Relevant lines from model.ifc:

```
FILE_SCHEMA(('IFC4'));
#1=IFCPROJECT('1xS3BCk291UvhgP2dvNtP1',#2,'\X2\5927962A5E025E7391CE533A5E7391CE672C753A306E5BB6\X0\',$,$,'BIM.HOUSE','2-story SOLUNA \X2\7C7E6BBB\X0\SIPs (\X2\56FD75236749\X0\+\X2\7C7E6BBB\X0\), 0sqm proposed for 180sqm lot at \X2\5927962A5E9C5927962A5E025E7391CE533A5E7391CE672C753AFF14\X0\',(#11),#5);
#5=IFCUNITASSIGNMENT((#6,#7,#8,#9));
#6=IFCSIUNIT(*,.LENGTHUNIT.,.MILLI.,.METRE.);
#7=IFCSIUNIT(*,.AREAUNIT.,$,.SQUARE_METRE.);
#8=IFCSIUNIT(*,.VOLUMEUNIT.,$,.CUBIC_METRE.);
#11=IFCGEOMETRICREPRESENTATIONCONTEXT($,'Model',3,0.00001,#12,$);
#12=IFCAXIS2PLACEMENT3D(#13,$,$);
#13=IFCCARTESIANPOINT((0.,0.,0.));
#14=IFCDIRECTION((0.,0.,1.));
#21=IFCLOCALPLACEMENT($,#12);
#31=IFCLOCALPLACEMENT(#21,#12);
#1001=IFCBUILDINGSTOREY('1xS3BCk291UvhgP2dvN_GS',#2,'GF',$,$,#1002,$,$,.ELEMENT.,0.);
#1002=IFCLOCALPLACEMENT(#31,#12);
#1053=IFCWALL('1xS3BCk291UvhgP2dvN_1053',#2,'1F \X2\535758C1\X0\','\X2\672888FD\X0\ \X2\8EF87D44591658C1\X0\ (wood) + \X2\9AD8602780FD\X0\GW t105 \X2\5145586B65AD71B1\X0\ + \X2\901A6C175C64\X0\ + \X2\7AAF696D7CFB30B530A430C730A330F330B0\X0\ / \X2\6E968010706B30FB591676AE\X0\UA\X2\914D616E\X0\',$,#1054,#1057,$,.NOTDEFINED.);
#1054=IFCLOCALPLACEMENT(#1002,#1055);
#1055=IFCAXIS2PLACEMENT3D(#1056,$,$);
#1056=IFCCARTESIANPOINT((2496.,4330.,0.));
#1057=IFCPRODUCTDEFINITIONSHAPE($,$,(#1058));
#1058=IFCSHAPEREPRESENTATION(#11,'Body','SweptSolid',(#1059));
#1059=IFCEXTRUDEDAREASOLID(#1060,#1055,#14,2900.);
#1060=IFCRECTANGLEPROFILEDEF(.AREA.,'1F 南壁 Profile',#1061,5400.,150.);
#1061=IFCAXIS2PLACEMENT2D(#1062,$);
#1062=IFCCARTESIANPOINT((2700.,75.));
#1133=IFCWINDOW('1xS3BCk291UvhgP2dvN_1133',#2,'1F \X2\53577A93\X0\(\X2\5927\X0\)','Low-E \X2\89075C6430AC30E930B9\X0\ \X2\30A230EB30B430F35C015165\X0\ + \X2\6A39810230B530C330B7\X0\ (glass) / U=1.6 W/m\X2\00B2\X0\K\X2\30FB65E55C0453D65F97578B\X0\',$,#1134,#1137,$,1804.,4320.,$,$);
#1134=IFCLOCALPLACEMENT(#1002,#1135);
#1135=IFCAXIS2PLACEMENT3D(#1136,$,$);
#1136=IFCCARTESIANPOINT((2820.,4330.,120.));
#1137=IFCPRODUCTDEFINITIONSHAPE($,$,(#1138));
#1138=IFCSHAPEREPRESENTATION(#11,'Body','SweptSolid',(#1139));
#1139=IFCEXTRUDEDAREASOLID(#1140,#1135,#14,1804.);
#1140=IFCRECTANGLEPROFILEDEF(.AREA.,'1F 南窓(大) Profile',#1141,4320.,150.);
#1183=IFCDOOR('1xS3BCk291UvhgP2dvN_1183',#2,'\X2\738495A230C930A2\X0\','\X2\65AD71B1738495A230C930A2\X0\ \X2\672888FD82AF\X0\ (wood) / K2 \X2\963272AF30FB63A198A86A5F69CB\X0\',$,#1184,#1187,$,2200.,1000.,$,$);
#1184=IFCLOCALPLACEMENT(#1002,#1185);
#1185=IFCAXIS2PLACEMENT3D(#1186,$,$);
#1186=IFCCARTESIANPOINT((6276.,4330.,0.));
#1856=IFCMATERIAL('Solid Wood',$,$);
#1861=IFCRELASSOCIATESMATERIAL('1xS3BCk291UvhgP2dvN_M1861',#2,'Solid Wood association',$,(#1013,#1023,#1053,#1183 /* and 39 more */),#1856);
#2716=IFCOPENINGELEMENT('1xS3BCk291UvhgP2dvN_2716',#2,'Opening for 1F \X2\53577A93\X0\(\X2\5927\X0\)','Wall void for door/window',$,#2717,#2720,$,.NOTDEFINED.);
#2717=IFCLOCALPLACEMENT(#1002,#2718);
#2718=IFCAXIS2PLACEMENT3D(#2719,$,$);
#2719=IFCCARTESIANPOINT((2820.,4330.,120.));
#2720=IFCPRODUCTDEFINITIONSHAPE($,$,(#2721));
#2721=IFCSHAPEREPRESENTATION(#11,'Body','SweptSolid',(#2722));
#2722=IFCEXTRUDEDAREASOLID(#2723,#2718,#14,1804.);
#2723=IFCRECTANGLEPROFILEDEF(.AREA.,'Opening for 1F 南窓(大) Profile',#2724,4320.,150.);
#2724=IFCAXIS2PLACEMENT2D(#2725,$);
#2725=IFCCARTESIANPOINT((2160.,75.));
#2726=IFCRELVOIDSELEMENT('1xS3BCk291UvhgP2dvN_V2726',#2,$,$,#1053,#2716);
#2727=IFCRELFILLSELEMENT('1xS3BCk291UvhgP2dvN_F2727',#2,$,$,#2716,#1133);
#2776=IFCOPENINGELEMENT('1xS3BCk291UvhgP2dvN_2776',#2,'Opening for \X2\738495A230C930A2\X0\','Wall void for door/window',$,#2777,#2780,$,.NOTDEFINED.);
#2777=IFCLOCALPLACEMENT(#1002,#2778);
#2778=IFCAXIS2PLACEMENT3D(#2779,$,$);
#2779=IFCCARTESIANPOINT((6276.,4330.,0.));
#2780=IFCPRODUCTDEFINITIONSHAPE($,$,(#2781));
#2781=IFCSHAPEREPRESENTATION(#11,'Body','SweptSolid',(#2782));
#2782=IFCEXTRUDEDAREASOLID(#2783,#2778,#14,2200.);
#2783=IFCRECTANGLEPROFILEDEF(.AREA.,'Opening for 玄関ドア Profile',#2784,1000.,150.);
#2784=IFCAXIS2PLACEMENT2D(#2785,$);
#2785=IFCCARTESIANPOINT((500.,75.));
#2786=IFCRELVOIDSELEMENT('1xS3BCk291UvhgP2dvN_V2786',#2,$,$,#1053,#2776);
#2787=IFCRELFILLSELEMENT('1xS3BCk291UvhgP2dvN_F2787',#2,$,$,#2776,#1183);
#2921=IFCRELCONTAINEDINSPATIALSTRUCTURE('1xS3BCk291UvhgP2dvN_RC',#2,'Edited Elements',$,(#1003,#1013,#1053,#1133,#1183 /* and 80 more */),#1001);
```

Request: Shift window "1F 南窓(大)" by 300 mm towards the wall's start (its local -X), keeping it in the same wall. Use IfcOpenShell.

```python
import ifcopenshell
import ifcopenshell.api.geometry
import ifcopenshell.util.placement
import ifcopenshell.util.unit

model = ifcopenshell.open("model.ifc")
unit_scale = ifcopenshell.util.unit.calculate_unit_scale(model)

window = model.by_id(1133)
opening = window.FillsVoids[0].RelatingOpeningElement
wall = opening.VoidsElements[0].RelatingBuildingElement

wall_matrix = ifcopenshell.util.placement.get_local_placement(wall.ObjectPlacement)
shift = wall_matrix[:3, 0] * -0.3 / unit_scale
before = ifcopenshell.util.placement.get_local_placement(window.ObjectPlacement)[:3, 3].copy()

# The window is not placed relative to its opening, so move both.
for product in (opening, window):
    matrix = ifcopenshell.util.placement.get_local_placement(product.ObjectPlacement)
    matrix[:3, 3] += shift
    ifcopenshell.api.geometry.edit_object_placement(model, product=product, matrix=matrix, is_si=False)

after = ifcopenshell.util.placement.get_local_placement(window.ObjectPlacement)[:3, 3]
print("window moved by", (after - before).round(3) + 0.0)

model.write("model_v2.ifc")
```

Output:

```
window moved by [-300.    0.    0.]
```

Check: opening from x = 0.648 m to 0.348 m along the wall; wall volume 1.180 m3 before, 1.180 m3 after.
